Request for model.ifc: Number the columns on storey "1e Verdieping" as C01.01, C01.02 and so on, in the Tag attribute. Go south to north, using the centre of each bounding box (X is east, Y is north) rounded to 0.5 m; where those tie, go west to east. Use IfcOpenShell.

First a look at what the model holds.

```python
import ifcopenshell
import ifcopenshell.util.element
import ifcopenshell.util.placement

model = ifcopenshell.open("model.ifc")
print(model.schema)
storey = next(s for s in model.by_type("IfcBuildingStorey") if s.Name == "1e Verdieping")
columns = [e for e in ifcopenshell.util.element.get_decomposition(storey) if e.is_a("IfcColumn")]
for e in sorted(columns, key=lambda e: e.id()):
    origin = ifcopenshell.util.placement.get_local_placement(e.ObjectPlacement)[:3, 3]
    print(e.id(), e.Tag, e.Name, origin.round(2) + 0.0, sep=" | ")
```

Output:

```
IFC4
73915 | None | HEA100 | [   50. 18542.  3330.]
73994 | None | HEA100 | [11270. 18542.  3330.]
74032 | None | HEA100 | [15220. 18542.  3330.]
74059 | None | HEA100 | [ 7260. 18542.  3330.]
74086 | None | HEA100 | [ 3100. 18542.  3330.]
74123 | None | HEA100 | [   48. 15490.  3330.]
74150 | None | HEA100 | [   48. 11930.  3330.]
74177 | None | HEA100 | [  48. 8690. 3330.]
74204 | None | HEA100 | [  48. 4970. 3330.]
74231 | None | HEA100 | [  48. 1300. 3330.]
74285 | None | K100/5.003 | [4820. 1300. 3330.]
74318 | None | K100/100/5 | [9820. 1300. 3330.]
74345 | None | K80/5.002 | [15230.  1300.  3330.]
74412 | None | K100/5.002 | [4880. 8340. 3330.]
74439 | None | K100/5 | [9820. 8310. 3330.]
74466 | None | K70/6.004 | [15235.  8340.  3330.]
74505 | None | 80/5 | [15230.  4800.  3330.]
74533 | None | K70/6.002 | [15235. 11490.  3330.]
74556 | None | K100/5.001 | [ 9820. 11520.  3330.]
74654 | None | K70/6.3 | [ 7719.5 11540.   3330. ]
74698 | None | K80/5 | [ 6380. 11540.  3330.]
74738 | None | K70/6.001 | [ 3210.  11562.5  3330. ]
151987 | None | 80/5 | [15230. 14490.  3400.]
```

```python
import ifcopenshell
import ifcopenshell.geom
import ifcopenshell.util.element
import ifcopenshell.util.shape

model = ifcopenshell.open("model.ifc")
settings = ifcopenshell.geom.settings()
settings.set("use-world-coords", True)


def centre(element):
    shape = ifcopenshell.geom.create_shape(settings, element)
    return ifcopenshell.util.shape.get_bbox_centroid(shape.geometry)


storey = next(s for s in model.by_type("IfcBuildingStorey") if s.Name == "1e Verdieping")
columns = [e for e in ifcopenshell.util.element.get_decomposition(storey) if e.is_a("IfcColumn")]

# Insertion points can sit at a corner or the storey origin, so sort by the geometry (in metres).
centres = {e: centre(e) for e in columns}
columns.sort(key=lambda e: (round(centres[e][1] / 0.5), centres[e][0]))

for i, e in enumerate(columns, start=1):
    number = f"C01.{i:02d}"
    e.Tag = number
    print(e.id(), number)

model.write("model_edited.ifc")
```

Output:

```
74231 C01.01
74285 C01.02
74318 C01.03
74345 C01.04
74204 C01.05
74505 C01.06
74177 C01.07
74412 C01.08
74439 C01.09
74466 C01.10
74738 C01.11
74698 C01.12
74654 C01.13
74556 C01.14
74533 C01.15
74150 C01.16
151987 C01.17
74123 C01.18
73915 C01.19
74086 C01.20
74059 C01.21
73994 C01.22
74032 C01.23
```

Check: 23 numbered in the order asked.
